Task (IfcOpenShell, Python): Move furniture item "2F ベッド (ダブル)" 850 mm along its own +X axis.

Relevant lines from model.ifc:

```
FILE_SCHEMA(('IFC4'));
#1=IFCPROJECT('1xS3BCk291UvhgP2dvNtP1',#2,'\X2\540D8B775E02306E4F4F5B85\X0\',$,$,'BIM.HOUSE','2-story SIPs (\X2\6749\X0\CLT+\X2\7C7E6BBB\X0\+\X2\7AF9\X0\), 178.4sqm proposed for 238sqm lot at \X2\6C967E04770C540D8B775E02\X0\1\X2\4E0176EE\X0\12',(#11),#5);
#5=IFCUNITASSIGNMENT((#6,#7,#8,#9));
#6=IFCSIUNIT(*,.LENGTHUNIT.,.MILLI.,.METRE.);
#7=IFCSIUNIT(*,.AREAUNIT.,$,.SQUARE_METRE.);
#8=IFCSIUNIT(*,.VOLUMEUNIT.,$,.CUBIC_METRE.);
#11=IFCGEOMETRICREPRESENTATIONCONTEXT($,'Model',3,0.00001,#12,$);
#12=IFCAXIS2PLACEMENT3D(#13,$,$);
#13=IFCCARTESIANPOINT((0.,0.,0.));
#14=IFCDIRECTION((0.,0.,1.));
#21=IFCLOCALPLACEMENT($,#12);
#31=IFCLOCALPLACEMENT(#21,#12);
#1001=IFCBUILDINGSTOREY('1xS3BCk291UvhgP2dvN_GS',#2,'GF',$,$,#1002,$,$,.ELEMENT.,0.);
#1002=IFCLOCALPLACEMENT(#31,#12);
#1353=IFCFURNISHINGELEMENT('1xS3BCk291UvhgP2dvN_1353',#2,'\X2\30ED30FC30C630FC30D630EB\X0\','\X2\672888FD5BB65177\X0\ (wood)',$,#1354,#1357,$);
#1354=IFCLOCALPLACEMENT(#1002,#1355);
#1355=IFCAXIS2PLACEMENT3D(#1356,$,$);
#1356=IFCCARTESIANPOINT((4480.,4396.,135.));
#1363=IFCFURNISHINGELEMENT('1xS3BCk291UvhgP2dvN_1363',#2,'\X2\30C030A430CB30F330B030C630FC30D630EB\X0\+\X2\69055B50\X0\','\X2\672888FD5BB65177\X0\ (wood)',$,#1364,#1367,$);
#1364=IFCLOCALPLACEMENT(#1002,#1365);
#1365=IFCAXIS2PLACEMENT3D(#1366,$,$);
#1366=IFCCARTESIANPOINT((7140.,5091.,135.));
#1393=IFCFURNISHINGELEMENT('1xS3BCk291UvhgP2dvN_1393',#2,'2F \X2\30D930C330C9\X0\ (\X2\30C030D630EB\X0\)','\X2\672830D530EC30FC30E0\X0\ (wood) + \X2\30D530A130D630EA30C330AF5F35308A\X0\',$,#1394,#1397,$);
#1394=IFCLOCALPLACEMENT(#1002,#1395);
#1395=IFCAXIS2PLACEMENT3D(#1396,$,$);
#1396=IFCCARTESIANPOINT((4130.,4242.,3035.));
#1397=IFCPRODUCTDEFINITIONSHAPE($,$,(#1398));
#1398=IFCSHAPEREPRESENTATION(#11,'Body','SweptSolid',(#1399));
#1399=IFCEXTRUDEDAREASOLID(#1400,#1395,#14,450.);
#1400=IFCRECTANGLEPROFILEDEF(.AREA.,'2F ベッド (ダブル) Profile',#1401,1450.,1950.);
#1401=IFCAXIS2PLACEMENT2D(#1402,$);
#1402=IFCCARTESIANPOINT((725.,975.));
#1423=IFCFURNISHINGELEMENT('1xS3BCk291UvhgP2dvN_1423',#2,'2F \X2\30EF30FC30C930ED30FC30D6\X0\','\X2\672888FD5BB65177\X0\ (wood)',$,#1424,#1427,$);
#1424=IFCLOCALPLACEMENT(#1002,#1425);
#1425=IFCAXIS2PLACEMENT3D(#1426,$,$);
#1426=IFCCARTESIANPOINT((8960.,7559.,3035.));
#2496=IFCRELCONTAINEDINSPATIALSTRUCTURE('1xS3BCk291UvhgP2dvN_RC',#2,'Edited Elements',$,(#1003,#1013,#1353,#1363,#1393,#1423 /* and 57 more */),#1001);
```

```python
import ifcopenshell
import ifcopenshell.api.geometry
import ifcopenshell.util.placement

model = ifcopenshell.open("model.ifc")

item = model.by_id(1393)
matrix = ifcopenshell.util.placement.get_local_placement(item.ObjectPlacement)
matrix[:3, 3] += matrix[:3, 0] * 850.0
ifcopenshell.api.geometry.edit_object_placement(model, product=item, matrix=matrix, is_si=False)

print(ifcopenshell.util.placement.get_local_placement(item.ObjectPlacement).round(3) + 0.0)

model.write("model_v2.ifc")
```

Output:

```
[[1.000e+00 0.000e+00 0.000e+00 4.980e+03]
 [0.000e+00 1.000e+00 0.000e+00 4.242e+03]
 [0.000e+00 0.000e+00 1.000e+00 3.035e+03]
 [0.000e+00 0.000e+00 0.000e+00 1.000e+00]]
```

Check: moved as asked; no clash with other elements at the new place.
